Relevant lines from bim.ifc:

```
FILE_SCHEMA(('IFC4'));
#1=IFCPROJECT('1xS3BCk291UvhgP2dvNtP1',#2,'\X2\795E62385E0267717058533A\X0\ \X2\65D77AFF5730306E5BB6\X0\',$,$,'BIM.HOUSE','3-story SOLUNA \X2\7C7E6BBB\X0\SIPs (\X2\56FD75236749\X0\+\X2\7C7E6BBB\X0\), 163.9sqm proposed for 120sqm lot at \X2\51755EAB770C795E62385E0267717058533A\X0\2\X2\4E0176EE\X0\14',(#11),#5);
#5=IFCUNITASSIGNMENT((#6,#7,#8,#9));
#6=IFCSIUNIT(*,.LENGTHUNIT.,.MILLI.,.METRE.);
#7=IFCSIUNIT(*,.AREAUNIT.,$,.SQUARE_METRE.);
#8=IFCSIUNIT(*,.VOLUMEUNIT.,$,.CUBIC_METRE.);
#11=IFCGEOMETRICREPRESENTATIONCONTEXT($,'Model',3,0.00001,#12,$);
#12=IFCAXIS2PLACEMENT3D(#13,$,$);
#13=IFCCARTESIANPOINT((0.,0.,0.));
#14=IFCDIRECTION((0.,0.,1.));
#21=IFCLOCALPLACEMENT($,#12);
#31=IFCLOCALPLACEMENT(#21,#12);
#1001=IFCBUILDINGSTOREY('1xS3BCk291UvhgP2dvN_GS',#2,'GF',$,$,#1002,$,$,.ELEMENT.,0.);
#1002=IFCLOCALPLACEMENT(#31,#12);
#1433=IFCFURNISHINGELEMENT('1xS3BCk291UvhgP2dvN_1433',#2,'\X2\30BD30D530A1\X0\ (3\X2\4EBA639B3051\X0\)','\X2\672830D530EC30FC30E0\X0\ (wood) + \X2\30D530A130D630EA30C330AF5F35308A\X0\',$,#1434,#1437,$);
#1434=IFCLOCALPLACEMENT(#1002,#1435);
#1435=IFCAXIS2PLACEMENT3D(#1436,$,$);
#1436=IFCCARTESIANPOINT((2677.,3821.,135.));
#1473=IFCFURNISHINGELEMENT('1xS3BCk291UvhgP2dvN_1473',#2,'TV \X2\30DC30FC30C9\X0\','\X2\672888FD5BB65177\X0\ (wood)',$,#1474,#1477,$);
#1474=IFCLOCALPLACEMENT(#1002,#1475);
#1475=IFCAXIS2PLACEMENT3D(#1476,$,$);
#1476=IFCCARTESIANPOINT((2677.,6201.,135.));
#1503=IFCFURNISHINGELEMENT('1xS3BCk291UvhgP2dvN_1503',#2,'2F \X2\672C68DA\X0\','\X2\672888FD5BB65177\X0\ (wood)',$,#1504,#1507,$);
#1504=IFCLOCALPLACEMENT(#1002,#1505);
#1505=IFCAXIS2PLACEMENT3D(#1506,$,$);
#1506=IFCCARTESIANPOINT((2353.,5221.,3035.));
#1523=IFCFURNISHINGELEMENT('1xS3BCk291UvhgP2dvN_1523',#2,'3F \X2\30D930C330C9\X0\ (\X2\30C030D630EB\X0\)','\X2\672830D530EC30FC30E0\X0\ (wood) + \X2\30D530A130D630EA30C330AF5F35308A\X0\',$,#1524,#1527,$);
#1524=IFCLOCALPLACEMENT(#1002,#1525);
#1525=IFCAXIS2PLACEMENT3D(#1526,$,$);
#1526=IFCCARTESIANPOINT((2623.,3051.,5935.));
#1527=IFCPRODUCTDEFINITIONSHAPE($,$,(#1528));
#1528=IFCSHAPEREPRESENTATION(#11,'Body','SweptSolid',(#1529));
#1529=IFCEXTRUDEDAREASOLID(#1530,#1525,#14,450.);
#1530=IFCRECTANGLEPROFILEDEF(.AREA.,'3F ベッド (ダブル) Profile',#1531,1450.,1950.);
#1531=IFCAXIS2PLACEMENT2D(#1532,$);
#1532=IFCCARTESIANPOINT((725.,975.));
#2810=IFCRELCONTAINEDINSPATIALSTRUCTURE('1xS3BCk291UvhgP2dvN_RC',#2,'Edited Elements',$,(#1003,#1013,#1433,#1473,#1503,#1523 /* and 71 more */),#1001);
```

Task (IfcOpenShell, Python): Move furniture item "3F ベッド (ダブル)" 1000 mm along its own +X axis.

```python
import ifcopenshell
import ifcopenshell.api.geometry
import ifcopenshell.util.placement
import ifcopenshell.util.unit

model = ifcopenshell.open("bim.ifc")
unit_scale = ifcopenshell.util.unit.calculate_unit_scale(model)

item = model.by_guid("1xS3BCk291UvhgP2dvN_1523")
matrix = ifcopenshell.util.placement.get_local_placement(item.ObjectPlacement)
matrix[:3, 3] += matrix[:3, 0] * 1 / unit_scale
ifcopenshell.api.geometry.edit_object_placement(model, product=item, matrix=matrix, is_si=False)

print(ifcopenshell.util.placement.get_local_placement(item.ObjectPlacement).round(3) + 0.0)

model.write("bim_edited.ifc")
```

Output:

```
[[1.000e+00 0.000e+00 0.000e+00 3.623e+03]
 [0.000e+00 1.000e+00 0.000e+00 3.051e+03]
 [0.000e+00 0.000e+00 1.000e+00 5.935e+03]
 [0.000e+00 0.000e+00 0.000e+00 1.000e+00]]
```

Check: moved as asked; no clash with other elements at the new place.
